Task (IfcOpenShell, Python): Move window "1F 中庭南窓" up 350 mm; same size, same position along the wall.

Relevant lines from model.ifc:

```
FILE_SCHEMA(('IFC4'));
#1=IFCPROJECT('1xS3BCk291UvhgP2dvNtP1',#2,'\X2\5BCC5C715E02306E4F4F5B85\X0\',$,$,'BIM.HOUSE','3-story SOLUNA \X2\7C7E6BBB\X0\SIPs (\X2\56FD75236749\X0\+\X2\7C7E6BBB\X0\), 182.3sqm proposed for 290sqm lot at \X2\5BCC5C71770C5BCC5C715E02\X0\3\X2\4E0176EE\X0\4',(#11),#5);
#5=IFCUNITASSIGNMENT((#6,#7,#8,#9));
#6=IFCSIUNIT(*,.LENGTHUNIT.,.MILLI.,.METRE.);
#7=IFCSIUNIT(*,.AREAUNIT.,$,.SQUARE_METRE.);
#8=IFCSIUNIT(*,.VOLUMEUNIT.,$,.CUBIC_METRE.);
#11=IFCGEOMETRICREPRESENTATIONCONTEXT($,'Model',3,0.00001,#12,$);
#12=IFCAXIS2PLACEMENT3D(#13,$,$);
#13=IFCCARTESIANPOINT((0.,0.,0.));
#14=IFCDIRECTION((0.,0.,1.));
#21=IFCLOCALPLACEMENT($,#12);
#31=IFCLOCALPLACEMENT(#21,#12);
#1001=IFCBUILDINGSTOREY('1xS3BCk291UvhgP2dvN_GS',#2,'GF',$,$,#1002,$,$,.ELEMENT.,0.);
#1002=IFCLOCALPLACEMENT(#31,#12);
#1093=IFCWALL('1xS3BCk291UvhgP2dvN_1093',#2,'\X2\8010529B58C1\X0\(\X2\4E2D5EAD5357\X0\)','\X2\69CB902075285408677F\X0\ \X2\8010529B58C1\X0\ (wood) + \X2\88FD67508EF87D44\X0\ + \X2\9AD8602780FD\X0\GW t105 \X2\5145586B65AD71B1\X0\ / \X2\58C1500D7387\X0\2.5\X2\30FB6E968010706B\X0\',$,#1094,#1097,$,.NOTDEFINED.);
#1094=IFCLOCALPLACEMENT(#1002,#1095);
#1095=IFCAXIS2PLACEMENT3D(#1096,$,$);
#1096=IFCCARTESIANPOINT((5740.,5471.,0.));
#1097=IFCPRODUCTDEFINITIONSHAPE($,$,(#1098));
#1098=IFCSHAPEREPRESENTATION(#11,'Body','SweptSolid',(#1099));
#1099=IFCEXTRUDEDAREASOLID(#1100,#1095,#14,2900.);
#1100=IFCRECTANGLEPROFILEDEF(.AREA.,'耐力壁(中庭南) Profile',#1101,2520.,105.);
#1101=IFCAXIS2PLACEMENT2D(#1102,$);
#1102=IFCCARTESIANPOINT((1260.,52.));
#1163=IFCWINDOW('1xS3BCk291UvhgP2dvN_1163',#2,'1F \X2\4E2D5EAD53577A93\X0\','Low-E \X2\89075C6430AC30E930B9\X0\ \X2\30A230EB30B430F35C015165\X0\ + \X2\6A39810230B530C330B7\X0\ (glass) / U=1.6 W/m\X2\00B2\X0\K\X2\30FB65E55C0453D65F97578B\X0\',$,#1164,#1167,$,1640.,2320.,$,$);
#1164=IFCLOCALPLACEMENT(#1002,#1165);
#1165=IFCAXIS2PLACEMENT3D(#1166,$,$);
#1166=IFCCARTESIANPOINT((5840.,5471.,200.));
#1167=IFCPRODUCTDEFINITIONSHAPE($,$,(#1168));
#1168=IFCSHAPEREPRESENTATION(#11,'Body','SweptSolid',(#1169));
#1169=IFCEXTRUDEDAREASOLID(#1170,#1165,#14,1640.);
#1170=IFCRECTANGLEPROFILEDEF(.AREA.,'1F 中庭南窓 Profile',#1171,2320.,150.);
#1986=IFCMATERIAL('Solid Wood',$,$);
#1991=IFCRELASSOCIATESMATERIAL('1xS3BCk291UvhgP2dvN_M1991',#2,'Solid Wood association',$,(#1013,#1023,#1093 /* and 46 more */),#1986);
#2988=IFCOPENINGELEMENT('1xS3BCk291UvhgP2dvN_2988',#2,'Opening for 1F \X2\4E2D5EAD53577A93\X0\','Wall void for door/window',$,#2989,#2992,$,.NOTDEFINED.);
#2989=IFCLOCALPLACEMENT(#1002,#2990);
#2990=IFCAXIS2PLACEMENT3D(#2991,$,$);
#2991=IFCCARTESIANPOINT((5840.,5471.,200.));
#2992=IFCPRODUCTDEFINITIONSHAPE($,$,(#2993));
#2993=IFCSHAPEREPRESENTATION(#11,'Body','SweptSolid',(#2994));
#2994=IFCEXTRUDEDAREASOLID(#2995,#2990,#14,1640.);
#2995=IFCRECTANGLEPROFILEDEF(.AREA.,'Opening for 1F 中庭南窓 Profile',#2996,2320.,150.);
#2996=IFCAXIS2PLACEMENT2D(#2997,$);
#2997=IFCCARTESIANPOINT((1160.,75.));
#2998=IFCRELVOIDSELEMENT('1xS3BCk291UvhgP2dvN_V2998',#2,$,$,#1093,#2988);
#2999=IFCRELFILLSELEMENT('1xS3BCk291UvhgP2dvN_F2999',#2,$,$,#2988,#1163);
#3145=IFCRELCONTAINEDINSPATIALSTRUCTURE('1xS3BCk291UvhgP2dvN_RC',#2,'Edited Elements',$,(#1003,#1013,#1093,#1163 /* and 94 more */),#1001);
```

```python
import numpy as np
import ifcopenshell
import ifcopenshell.api.geometry
import ifcopenshell.util.placement
import ifcopenshell.util.unit

model = ifcopenshell.open("model.ifc")
unit_scale = ifcopenshell.util.unit.calculate_unit_scale(model)

window = model.by_guid("1xS3BCk291UvhgP2dvN_1163")
opening = window.FillsVoids[0].RelatingOpeningElement
dz = 350.0

shift = np.array([0.0, 0.0, dz])
# The window is not placed relative to its opening, so move both.
for product in (opening, window):
    matrix = ifcopenshell.util.placement.get_local_placement(product.ObjectPlacement)
    matrix[:3, 3] += shift
    ifcopenshell.api.geometry.edit_object_placement(model, product=product, matrix=matrix, is_si=False)

print(f"moved by {dz * unit_scale:+.3f} m")

model.write("model_v2.ifc")
```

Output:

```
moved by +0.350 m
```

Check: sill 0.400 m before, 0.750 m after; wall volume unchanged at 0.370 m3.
